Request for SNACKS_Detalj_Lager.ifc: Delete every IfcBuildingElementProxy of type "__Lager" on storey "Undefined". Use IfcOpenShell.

First a look at what the model holds.

```python
import ifcopenshell
import ifcopenshell.util.element

model = ifcopenshell.open("SNACKS_Detalj_Lager.ifc")
print(model.schema)
storey = next(s for s in model.by_type("IfcBuildingStorey") if s.Name == "Undefined")
proxies = [e for e in ifcopenshell.util.element.get_decomposition(storey) if e.is_a("IfcBuildingElementProxy")]
seen = {}
for e in proxies:
    element_type = ifcopenshell.util.element.get_type(e)
    name = element_type.Name if element_type not in (None, e) else None
    seen[name] = seen.get(name, 0) + 1
for name, count in sorted(seen.items(), key=str):
    print(count, "x", name)
```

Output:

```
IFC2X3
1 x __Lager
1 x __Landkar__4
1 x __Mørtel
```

```python
import ifcopenshell
import ifcopenshell.api.root
import ifcopenshell.util.element

model = ifcopenshell.open("SNACKS_Detalj_Lager.ifc")

storey = next(s for s in model.by_type("IfcBuildingStorey") if s.Name == "Undefined")
proxies = [e for e in ifcopenshell.util.element.get_decomposition(storey) if e.is_a("IfcBuildingElementProxy")]
targets = [e for e in proxies if (t := ifcopenshell.util.element.get_type(e)) not in (None, e) and t.Name == "__Lager"]

for e in targets:
    ifcopenshell.api.root.remove_product(model, product=e)
print(len(targets), "removed")

model.write("SNACKS_Detalj_Lager_v2.ifc")
```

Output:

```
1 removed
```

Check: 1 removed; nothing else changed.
